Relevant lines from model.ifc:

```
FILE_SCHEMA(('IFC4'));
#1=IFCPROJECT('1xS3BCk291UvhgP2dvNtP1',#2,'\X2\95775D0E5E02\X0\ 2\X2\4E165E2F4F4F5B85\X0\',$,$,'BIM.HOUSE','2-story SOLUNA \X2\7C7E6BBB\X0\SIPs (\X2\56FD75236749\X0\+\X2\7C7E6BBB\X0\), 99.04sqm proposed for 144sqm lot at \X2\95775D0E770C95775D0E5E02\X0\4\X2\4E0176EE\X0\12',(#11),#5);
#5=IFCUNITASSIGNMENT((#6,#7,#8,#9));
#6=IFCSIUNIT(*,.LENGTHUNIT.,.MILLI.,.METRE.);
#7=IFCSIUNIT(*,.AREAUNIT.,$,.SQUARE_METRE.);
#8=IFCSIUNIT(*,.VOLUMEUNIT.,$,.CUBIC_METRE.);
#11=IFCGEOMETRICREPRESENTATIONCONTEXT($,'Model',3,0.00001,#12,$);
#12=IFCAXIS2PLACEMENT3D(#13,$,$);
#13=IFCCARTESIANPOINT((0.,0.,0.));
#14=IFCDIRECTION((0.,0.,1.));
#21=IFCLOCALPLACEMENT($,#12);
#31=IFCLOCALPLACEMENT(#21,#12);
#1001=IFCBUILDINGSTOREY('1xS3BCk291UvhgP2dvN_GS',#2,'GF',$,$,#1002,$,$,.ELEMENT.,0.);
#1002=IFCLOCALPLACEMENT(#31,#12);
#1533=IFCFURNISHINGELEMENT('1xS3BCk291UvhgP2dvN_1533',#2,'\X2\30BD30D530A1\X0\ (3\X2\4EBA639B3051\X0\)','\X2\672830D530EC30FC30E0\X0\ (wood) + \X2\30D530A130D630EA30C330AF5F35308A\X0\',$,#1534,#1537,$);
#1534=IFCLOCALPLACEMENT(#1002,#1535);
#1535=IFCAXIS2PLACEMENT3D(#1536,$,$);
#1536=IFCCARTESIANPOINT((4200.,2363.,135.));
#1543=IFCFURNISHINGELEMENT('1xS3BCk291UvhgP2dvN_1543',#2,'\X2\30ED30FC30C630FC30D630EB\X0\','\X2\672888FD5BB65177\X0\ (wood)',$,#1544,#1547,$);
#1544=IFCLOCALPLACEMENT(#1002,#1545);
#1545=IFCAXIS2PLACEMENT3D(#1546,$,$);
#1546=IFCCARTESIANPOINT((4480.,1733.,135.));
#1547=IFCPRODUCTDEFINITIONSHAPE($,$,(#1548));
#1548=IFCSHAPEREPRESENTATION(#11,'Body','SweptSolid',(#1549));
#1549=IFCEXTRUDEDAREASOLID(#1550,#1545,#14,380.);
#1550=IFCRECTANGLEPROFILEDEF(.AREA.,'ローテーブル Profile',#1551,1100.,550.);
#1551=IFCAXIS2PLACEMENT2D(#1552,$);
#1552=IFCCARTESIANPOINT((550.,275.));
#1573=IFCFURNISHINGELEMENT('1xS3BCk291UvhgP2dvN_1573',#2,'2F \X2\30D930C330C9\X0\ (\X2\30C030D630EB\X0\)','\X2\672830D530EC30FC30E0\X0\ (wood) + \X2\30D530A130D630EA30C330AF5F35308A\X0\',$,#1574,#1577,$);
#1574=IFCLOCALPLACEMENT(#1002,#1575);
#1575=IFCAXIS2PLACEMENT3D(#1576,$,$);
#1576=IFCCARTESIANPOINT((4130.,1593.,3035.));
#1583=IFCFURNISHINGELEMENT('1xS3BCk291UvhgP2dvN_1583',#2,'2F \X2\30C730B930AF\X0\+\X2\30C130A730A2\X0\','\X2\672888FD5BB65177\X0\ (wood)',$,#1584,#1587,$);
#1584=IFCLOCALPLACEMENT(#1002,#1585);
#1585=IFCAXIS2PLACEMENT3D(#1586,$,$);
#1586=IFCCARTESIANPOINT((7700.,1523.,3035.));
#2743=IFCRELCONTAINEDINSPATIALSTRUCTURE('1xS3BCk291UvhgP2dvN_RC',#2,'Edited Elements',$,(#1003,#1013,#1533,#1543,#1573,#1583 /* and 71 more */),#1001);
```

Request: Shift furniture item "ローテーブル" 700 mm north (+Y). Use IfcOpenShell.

```python
import ifcopenshell
import ifcopenshell.api.geometry
import ifcopenshell.util.placement
import ifcopenshell.util.unit

model = ifcopenshell.open("model.ifc")
unit_scale = ifcopenshell.util.unit.calculate_unit_scale(model)

item = model.by_guid("1xS3BCk291UvhgP2dvN_1543")
matrix = ifcopenshell.util.placement.get_local_placement(item.ObjectPlacement)
matrix[1, 3] += 0.7 / unit_scale
ifcopenshell.api.geometry.edit_object_placement(model, product=item, matrix=matrix, is_si=False)

print(ifcopenshell.util.placement.get_local_placement(item.ObjectPlacement).round(3) + 0.0)

model.write("model_rev.ifc")
```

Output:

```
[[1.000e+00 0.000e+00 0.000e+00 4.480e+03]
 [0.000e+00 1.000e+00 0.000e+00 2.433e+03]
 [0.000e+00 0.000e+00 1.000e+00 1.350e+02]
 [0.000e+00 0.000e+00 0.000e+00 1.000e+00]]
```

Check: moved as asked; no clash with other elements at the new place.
